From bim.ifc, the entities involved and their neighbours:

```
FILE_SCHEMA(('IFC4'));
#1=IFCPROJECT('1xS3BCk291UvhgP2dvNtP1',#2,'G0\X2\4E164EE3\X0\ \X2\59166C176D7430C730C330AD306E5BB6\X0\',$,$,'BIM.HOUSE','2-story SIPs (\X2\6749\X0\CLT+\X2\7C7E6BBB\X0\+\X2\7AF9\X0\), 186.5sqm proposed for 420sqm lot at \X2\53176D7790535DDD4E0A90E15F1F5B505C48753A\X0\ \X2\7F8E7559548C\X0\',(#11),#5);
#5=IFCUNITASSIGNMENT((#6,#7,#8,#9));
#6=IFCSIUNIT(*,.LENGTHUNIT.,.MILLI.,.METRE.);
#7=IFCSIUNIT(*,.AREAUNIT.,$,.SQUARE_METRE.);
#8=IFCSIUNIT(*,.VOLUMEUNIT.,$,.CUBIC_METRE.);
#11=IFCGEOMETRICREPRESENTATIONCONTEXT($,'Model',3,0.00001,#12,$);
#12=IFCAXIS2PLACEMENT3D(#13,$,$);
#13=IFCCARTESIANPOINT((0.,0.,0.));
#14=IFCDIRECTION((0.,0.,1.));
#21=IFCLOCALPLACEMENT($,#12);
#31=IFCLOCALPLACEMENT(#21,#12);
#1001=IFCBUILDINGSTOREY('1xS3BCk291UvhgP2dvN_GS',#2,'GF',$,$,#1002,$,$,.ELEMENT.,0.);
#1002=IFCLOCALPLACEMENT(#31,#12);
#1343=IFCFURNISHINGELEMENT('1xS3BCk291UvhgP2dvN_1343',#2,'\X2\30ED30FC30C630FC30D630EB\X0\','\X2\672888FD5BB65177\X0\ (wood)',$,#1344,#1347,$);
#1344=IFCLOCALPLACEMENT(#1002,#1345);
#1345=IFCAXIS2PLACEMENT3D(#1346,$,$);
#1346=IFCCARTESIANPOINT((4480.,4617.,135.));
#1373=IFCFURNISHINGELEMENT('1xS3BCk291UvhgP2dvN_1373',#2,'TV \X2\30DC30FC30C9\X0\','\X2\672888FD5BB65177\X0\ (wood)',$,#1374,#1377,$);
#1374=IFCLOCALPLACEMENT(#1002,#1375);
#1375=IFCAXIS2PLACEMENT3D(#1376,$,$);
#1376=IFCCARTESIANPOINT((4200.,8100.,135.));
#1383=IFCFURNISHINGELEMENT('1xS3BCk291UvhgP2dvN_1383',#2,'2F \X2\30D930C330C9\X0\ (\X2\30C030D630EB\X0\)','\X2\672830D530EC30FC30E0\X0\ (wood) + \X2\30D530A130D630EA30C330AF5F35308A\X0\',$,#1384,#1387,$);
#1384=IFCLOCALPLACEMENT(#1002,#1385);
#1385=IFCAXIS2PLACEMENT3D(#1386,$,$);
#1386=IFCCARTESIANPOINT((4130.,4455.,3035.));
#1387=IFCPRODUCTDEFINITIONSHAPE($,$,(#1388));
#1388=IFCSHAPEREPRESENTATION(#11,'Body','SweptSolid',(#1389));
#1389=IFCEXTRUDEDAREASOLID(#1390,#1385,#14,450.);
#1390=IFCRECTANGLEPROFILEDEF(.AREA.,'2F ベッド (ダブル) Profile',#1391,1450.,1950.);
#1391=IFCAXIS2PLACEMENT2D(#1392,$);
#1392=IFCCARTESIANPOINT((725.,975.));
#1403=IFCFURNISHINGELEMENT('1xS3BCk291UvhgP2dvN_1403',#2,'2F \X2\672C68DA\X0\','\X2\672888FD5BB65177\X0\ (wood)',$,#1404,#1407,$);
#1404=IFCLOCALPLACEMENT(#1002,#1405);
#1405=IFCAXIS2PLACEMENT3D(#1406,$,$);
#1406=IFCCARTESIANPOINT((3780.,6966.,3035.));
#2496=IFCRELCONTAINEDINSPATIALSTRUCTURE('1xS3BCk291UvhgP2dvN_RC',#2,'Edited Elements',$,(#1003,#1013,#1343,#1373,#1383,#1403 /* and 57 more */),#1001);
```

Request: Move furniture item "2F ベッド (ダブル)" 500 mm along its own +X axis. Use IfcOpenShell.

```python
import ifcopenshell
import ifcopenshell.api.geometry
import ifcopenshell.util.placement
import ifcopenshell.util.unit

model = ifcopenshell.open("bim.ifc")
unit_scale = ifcopenshell.util.unit.calculate_unit_scale(model)

item = model.by_guid("1xS3BCk291UvhgP2dvN_1383")
matrix = ifcopenshell.util.placement.get_local_placement(item.ObjectPlacement)
matrix[:3, 3] += matrix[:3, 0] * 0.5 / unit_scale
ifcopenshell.api.geometry.edit_object_placement(model, product=item, matrix=matrix, is_si=False)

print(ifcopenshell.util.placement.get_local_placement(item.ObjectPlacement).round(3) + 0.0)

model.write("bim-out.ifc")
```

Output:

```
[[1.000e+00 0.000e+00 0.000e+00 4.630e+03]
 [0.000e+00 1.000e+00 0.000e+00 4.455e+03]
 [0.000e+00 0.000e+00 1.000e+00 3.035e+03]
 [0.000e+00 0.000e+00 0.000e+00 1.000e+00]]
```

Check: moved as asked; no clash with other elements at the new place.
